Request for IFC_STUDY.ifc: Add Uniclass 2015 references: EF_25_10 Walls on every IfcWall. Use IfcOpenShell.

First a look at what the model holds.

```python
import ifcopenshell

model = ifcopenshell.open("IFC_STUDY.ifc")
print(model.schema)
print("classifications:", [c.Name for c in model.by_type("IfcClassification")])
for ifc_class in ("IfcDoor", "IfcRoof", "IfcStair", "IfcWall", "IfcWindow"):
    print(ifc_class, len(model.by_type(ifc_class)))
```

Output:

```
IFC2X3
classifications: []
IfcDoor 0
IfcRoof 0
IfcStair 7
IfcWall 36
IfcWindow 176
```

```python
import ifcopenshell
import ifcopenshell.api.classification

model = ifcopenshell.open("IFC_STUDY.ifc")

# IFC2X3 requires Source and Edition and has no link from the project to the system.
system = model.create_entity("IfcClassification", Source="NBS", Edition="2015", Name="Uniclass 2015")

codes = {
    "IfcWall": ("EF_25_10", "Walls"),
}
for ifc_class, (code, name) in codes.items():
    products = model.by_type(ifc_class)
    ifcopenshell.api.classification.add_reference(
        model, products=products, classification=system, identification=code, name=name
    )
    print(code, len(products))

model.write("IFC_STUDY_edited.ifc")
```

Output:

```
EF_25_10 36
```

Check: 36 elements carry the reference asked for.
